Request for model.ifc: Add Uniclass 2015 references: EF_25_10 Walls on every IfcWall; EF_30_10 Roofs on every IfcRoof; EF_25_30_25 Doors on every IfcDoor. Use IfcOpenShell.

First a look at what the model holds.

```python
import ifcopenshell

model = ifcopenshell.open("model.ifc")
print(model.schema)
print("classifications:", [c.Name for c in model.by_type("IfcClassification")])
for ifc_class in ("IfcDoor", "IfcRoof", "IfcStair", "IfcWall", "IfcWindow"):
    print(ifc_class, len(model.by_type(ifc_class)))
```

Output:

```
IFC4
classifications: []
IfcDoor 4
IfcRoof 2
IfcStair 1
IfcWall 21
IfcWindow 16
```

```python
import ifcopenshell
import ifcopenshell.api.classification

model = ifcopenshell.open("model.ifc")

system = ifcopenshell.api.classification.add_classification(model, classification="Uniclass 2015")

codes = {
    "IfcWall": ("EF_25_10", "Walls"),
    "IfcRoof": ("EF_30_10", "Roofs"),
    "IfcDoor": ("EF_25_30_25", "Doors"),
}
for ifc_class, (code, name) in codes.items():
    products = model.by_type(ifc_class)
    ifcopenshell.api.classification.add_reference(
        model, products=products, classification=system, identification=code, name=name
    )
    print(code, len(products))

model.write("model-out.ifc")
```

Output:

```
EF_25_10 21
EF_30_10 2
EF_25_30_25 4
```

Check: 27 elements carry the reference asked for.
